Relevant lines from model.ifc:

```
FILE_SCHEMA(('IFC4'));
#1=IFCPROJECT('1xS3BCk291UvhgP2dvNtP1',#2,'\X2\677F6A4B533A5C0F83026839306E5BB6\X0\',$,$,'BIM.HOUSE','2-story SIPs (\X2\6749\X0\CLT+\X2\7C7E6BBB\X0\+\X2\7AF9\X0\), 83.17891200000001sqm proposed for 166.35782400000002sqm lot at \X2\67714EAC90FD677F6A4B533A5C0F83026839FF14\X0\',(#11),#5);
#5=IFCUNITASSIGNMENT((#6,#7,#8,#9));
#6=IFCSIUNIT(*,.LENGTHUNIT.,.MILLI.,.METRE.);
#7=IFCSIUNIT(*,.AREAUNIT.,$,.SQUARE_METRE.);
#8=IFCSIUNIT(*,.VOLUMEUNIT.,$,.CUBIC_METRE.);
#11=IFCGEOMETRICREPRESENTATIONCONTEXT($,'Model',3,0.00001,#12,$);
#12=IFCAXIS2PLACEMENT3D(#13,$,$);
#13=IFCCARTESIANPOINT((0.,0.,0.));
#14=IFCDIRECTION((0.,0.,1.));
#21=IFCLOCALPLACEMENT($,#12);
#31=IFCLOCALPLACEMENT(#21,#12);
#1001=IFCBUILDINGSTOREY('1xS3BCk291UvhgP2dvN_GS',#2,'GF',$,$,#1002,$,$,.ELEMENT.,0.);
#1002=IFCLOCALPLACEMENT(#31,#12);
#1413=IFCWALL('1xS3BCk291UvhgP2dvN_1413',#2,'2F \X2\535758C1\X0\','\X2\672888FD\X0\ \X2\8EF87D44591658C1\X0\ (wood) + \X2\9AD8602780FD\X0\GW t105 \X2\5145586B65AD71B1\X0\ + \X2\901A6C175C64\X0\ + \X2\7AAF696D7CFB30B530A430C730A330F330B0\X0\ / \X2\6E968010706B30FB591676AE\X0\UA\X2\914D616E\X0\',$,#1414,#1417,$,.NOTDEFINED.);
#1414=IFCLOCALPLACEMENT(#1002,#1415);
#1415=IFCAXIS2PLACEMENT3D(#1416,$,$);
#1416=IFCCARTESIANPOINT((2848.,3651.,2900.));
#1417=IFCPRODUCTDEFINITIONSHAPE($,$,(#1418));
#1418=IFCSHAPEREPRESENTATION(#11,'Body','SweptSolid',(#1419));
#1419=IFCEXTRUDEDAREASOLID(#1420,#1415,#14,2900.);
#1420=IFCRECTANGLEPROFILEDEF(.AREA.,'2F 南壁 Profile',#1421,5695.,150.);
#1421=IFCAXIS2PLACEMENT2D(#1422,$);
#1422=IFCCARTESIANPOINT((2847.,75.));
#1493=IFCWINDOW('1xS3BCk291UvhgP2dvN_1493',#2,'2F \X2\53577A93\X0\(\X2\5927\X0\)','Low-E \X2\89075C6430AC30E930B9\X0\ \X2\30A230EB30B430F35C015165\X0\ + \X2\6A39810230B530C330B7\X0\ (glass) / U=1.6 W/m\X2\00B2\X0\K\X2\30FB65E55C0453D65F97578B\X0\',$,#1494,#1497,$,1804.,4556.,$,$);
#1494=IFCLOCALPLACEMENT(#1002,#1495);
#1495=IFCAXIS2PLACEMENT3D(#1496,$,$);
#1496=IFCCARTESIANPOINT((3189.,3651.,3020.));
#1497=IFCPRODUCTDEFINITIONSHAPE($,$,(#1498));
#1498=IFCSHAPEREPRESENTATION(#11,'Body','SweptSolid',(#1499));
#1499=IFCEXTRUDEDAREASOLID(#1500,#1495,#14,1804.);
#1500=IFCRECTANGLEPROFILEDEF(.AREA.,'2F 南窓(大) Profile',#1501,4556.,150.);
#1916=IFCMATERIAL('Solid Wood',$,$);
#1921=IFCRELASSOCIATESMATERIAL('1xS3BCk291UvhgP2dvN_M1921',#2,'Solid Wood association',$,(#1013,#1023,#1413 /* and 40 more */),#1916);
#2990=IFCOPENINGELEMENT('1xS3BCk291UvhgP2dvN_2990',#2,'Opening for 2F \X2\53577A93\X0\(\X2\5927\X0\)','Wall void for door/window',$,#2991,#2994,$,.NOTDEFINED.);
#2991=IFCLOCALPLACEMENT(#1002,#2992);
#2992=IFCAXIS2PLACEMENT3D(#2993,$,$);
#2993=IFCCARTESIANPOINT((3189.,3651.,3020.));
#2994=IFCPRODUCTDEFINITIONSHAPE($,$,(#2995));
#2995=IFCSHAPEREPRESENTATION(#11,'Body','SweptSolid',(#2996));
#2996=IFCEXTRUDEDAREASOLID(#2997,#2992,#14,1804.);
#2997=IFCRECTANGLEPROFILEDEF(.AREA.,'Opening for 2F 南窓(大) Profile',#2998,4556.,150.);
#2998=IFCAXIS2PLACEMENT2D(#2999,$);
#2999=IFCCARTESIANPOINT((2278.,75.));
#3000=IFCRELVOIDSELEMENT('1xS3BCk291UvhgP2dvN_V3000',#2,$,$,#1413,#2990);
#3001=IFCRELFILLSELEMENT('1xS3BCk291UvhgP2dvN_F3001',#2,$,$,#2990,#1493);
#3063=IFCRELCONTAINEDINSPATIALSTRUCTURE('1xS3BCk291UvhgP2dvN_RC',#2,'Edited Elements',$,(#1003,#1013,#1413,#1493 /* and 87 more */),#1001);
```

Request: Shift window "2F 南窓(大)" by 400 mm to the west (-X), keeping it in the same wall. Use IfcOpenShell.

```python
import ifcopenshell
import ifcopenshell.api.geometry
import ifcopenshell.util.placement

model = ifcopenshell.open("model.ifc")

window = model.by_guid("1xS3BCk291UvhgP2dvN_1493")
opening = window.FillsVoids[0].RelatingOpeningElement
wall = opening.VoidsElements[0].RelatingBuildingElement

wall_matrix = ifcopenshell.util.placement.get_local_placement(wall.ObjectPlacement)
shift = wall_matrix[:3, 0] * -400.0
before = ifcopenshell.util.placement.get_local_placement(window.ObjectPlacement)[:3, 3].copy()

# The window is not placed relative to its opening, so move both.
for product in (opening, window):
    matrix = ifcopenshell.util.placement.get_local_placement(product.ObjectPlacement)
    matrix[:3, 3] += shift
    ifcopenshell.api.geometry.edit_object_placement(model, product=product, matrix=matrix, is_si=False)

after = ifcopenshell.util.placement.get_local_placement(window.ObjectPlacement)[:3, 3]
print("window moved by", (after - before).round(3) + 0.0)

model.write("model-out.ifc")
```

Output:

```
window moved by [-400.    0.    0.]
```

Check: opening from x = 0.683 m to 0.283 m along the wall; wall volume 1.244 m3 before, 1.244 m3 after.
